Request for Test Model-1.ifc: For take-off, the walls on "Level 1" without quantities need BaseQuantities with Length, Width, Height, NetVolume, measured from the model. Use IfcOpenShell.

First a look at what the model holds.

```python
import ifcopenshell
import ifcopenshell.util.element
import ifcopenshell.util.unit

model = ifcopenshell.open("Test Model-1.ifc")
print(model.schema)
for unit_type in ("LENGTHUNIT", "AREAUNIT", "VOLUMEUNIT"):
    print(unit_type, ifcopenshell.util.unit.calculate_unit_scale(model, unit_type))
storey = next(s for s in model.by_type("IfcBuildingStorey") if s.Name == "Level 1")
walls = [e for e in ifcopenshell.util.element.get_decomposition(storey) if e.is_a("IfcWall")]
for e in sorted(walls, key=lambda e: e.id()):
    print(e.id(), e.is_a(), e.Name, list(ifcopenshell.util.element.get_psets(e, qtos_only=True)), sep=" | ")
```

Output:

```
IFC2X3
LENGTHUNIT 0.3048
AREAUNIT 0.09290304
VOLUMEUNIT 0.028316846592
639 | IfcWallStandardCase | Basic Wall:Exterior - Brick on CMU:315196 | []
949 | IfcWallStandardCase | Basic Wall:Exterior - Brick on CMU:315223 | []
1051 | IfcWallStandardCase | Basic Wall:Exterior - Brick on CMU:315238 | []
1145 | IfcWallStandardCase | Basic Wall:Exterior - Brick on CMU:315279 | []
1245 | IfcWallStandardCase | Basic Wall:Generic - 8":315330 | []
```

```python
import ifcopenshell
import ifcopenshell.api.pset
import ifcopenshell.geom
import ifcopenshell.util.element
import ifcopenshell.util.shape
import ifcopenshell.util.unit

model = ifcopenshell.open("Test Model-1.ifc")
unit_scale = ifcopenshell.util.unit.calculate_unit_scale(model)
volume_scale = ifcopenshell.util.unit.calculate_unit_scale(model, "VOLUMEUNIT")
settings = ifcopenshell.geom.settings()

storey = next(s for s in model.by_type("IfcBuildingStorey") if s.Name == "Level 1")
walls = [e for e in ifcopenshell.util.element.get_decomposition(storey) if e.is_a("IfcWall")]

for e in sorted(walls, key=lambda e: e.id()):
    if ifcopenshell.util.element.get_psets(e, qtos_only=True, should_inherit=False):
        continue
    # Geometry comes back in metres, in the element's own axes.
    shape = ifcopenshell.geom.create_shape(settings, e)
    values = {
        "Length": ifcopenshell.util.shape.get_x(shape.geometry) / unit_scale,
        "Width": ifcopenshell.util.shape.get_y(shape.geometry) / unit_scale,
        "Height": ifcopenshell.util.shape.get_z(shape.geometry) / unit_scale,
        "NetVolume": ifcopenshell.util.shape.get_volume(shape.geometry) / volume_scale,
    }
    qto = ifcopenshell.api.pset.add_qto(model, product=e, name="BaseQuantities")
    ifcopenshell.api.pset.edit_qto(model, qto=qto, properties=values)
    print(e.id(), {k: round(v, 3) for k, v in values.items()})

model.write("Test Model-1_updated.ifc")
```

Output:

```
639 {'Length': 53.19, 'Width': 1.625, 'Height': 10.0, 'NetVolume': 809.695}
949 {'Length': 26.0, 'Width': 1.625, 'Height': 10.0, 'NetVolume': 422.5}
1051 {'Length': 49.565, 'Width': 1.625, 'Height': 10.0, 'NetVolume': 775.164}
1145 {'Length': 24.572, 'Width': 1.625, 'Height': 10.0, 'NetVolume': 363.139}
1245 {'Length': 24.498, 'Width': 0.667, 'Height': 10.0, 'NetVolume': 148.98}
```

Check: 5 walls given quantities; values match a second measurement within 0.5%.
